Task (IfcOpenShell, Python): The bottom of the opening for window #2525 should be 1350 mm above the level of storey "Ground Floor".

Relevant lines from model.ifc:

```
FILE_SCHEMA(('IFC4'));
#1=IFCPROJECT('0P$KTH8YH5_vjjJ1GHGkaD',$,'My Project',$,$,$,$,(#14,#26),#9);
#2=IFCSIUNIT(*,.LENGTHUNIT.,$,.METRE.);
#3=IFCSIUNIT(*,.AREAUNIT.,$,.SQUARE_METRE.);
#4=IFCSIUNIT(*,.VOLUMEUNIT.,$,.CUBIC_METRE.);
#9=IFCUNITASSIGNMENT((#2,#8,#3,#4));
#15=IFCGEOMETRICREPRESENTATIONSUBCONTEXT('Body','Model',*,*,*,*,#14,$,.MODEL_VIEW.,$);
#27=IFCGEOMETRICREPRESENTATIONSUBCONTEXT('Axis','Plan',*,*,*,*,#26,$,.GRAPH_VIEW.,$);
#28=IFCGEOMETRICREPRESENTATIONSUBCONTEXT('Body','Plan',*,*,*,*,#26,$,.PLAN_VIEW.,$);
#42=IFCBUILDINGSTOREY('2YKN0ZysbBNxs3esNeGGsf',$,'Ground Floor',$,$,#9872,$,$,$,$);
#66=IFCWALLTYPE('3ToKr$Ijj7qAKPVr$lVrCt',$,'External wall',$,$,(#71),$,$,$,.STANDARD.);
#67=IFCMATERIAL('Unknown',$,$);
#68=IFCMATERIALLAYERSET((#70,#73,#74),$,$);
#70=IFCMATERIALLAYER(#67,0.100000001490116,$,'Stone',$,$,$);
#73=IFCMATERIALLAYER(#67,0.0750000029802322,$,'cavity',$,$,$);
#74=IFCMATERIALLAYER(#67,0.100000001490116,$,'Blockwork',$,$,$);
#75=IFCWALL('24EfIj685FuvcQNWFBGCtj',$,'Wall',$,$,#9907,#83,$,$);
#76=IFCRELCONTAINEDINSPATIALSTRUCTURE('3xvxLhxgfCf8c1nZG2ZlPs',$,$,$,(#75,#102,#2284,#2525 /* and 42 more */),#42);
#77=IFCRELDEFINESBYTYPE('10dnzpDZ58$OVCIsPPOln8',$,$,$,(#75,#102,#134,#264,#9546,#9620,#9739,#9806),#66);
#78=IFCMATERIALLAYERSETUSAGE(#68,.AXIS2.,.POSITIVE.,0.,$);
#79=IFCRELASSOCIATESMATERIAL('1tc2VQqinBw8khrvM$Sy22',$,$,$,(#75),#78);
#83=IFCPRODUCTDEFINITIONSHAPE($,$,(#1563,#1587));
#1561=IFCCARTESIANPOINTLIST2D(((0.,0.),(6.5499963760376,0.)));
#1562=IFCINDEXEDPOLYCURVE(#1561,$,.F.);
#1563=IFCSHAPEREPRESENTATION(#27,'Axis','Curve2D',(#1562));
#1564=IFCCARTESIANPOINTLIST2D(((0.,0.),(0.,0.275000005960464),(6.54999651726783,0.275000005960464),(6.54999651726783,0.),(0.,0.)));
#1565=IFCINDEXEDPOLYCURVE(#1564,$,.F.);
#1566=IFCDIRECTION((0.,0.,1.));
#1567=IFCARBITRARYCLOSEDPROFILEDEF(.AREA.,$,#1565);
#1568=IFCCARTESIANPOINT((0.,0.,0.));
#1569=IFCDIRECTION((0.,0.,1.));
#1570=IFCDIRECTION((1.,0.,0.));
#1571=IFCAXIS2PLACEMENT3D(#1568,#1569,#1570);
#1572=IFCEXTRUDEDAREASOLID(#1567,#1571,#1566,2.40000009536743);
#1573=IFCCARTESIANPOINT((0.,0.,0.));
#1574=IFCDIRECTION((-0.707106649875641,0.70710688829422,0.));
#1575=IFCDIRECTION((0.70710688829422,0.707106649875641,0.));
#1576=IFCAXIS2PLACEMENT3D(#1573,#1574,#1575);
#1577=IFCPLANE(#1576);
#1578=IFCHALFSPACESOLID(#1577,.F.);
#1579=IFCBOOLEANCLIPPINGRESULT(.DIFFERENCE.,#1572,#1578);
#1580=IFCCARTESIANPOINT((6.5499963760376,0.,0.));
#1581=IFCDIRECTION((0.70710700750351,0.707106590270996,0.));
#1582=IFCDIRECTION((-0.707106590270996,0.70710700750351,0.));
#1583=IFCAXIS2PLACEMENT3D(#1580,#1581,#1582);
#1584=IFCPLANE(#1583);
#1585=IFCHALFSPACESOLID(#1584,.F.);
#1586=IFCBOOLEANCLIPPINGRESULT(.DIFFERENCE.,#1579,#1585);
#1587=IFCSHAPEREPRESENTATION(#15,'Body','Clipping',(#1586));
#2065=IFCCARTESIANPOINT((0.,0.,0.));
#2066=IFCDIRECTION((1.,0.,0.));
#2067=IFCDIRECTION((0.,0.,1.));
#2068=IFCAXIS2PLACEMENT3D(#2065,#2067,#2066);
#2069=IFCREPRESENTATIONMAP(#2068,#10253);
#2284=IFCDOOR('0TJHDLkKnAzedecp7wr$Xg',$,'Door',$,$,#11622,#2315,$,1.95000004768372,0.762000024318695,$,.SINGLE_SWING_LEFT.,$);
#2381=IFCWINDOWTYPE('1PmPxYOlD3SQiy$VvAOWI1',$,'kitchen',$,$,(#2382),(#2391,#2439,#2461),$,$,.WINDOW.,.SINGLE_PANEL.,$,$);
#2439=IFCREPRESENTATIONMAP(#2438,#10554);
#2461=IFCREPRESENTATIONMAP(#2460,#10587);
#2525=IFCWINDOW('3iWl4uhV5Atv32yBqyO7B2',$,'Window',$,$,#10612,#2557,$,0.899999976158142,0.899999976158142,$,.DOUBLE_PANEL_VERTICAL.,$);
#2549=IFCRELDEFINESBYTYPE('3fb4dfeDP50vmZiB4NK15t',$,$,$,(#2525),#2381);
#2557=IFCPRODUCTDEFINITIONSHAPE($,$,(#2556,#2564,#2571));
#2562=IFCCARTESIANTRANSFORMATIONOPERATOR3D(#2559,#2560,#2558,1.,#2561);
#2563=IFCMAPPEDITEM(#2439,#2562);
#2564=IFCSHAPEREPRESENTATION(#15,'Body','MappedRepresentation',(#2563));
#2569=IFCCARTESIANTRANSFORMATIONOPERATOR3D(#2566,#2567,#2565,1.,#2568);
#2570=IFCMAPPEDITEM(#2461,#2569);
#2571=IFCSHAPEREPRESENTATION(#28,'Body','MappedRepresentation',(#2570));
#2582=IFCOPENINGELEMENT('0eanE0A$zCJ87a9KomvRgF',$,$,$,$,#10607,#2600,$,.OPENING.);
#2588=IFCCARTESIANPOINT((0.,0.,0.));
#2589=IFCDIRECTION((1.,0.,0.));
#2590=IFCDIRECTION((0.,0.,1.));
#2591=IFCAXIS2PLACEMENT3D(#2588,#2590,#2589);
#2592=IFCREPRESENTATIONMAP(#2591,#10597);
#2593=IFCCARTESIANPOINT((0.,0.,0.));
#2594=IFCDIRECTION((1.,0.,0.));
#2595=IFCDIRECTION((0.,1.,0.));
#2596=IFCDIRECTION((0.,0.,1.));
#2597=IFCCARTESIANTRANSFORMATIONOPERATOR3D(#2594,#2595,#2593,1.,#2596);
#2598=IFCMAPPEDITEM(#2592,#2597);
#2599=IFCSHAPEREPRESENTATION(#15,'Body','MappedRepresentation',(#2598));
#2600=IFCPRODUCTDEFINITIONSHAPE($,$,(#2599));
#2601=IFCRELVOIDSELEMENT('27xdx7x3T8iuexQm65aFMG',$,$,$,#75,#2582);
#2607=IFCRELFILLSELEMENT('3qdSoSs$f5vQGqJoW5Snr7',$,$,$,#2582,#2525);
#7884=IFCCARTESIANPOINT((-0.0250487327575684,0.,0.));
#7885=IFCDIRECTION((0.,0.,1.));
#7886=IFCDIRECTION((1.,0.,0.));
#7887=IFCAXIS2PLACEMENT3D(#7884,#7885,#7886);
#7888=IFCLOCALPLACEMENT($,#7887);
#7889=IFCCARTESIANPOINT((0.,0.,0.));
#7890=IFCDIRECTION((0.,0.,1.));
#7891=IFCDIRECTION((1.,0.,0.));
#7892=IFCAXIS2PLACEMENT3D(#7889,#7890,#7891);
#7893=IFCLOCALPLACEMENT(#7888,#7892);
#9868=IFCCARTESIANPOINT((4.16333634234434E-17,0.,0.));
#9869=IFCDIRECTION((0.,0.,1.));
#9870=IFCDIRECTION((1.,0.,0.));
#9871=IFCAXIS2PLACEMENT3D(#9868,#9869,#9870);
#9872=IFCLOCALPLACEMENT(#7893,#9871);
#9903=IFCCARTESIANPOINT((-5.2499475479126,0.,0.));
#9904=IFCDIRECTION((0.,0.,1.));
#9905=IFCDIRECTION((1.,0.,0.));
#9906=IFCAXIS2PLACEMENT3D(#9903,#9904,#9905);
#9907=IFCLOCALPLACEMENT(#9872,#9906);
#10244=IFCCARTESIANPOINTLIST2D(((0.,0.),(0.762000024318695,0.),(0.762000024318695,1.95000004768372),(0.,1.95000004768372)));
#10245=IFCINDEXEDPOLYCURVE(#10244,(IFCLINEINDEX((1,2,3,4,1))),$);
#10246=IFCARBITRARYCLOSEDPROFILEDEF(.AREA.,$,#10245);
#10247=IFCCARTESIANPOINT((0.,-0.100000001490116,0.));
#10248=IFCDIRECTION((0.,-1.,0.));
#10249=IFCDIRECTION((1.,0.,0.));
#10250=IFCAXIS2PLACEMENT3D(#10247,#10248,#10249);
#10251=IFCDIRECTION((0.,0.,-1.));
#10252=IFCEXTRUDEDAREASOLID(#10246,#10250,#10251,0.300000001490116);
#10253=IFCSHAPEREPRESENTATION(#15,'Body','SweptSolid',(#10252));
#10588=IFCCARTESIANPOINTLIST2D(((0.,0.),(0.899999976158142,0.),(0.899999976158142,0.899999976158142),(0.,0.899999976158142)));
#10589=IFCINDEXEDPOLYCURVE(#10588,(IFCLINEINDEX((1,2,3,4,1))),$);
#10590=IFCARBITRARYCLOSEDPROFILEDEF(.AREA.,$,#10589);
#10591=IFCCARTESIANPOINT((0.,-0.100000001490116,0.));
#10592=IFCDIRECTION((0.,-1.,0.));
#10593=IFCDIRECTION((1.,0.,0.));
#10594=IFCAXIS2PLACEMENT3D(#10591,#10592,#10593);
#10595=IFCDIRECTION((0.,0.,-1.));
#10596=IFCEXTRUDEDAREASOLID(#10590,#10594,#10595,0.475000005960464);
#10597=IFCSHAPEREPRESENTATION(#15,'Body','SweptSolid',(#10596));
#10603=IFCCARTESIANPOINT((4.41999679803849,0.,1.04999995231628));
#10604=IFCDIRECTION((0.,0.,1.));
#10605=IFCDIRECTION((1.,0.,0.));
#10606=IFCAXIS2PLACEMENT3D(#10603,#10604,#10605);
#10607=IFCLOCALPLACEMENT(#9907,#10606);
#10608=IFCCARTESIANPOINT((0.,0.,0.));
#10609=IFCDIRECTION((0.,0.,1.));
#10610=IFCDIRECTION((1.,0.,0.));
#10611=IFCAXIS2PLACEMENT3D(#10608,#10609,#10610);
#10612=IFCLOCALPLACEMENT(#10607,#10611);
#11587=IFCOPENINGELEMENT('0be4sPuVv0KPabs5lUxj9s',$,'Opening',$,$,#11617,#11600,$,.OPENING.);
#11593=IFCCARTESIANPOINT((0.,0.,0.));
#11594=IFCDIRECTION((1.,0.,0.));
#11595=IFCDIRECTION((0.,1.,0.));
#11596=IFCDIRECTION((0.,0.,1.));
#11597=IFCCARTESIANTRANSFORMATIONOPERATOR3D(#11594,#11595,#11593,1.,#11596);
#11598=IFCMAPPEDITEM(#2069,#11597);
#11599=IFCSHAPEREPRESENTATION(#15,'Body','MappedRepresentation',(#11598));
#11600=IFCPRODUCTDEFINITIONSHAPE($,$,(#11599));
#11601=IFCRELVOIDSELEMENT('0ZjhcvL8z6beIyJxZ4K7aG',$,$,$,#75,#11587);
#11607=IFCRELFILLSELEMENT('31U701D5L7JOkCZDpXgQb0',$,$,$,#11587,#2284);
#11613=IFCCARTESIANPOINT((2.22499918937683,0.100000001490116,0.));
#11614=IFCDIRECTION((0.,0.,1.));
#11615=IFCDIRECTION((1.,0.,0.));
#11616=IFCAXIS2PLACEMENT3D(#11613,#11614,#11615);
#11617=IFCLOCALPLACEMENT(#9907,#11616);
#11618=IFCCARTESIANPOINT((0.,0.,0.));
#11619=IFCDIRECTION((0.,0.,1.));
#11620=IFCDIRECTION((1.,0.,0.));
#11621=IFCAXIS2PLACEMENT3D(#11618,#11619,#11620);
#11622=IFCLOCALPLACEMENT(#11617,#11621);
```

```python
import numpy as np
import ifcopenshell
import ifcopenshell.api.geometry
import ifcopenshell.geom
import ifcopenshell.util.element
import ifcopenshell.util.placement
import ifcopenshell.util.shape
import ifcopenshell.util.unit

model = ifcopenshell.open("model.ifc")
unit_scale = ifcopenshell.util.unit.calculate_unit_scale(model)

window = model.by_id(2525)
opening = window.FillsVoids[0].RelatingOpeningElement
storey = ifcopenshell.util.element.get_container(window, ifc_class="IfcBuildingStorey")
level = ifcopenshell.util.placement.get_local_placement(storey.ObjectPlacement)[2, 3]

# The opening's origin need not be at the sill, so measure its lowest point.
shape = ifcopenshell.geom.create_shape(ifcopenshell.geom.settings(), opening)
bottom = ifcopenshell.util.shape.get_shape_bottom_elevation(shape, shape.geometry) / unit_scale
dz = level + 1.35 / unit_scale - bottom

shift = np.array([0.0, 0.0, dz])
# The window is placed relative to its opening, so it follows when the opening moves.
matrix = ifcopenshell.util.placement.get_local_placement(opening.ObjectPlacement)
matrix[:3, 3] += shift
ifcopenshell.api.geometry.edit_object_placement(
    model, product=opening, matrix=matrix, is_si=False, should_transform_children=True
)

print(f"moved by {dz * unit_scale:+.3f} m")

model.write("model_edited.ifc")
```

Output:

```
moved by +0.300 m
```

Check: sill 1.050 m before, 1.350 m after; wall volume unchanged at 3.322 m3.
